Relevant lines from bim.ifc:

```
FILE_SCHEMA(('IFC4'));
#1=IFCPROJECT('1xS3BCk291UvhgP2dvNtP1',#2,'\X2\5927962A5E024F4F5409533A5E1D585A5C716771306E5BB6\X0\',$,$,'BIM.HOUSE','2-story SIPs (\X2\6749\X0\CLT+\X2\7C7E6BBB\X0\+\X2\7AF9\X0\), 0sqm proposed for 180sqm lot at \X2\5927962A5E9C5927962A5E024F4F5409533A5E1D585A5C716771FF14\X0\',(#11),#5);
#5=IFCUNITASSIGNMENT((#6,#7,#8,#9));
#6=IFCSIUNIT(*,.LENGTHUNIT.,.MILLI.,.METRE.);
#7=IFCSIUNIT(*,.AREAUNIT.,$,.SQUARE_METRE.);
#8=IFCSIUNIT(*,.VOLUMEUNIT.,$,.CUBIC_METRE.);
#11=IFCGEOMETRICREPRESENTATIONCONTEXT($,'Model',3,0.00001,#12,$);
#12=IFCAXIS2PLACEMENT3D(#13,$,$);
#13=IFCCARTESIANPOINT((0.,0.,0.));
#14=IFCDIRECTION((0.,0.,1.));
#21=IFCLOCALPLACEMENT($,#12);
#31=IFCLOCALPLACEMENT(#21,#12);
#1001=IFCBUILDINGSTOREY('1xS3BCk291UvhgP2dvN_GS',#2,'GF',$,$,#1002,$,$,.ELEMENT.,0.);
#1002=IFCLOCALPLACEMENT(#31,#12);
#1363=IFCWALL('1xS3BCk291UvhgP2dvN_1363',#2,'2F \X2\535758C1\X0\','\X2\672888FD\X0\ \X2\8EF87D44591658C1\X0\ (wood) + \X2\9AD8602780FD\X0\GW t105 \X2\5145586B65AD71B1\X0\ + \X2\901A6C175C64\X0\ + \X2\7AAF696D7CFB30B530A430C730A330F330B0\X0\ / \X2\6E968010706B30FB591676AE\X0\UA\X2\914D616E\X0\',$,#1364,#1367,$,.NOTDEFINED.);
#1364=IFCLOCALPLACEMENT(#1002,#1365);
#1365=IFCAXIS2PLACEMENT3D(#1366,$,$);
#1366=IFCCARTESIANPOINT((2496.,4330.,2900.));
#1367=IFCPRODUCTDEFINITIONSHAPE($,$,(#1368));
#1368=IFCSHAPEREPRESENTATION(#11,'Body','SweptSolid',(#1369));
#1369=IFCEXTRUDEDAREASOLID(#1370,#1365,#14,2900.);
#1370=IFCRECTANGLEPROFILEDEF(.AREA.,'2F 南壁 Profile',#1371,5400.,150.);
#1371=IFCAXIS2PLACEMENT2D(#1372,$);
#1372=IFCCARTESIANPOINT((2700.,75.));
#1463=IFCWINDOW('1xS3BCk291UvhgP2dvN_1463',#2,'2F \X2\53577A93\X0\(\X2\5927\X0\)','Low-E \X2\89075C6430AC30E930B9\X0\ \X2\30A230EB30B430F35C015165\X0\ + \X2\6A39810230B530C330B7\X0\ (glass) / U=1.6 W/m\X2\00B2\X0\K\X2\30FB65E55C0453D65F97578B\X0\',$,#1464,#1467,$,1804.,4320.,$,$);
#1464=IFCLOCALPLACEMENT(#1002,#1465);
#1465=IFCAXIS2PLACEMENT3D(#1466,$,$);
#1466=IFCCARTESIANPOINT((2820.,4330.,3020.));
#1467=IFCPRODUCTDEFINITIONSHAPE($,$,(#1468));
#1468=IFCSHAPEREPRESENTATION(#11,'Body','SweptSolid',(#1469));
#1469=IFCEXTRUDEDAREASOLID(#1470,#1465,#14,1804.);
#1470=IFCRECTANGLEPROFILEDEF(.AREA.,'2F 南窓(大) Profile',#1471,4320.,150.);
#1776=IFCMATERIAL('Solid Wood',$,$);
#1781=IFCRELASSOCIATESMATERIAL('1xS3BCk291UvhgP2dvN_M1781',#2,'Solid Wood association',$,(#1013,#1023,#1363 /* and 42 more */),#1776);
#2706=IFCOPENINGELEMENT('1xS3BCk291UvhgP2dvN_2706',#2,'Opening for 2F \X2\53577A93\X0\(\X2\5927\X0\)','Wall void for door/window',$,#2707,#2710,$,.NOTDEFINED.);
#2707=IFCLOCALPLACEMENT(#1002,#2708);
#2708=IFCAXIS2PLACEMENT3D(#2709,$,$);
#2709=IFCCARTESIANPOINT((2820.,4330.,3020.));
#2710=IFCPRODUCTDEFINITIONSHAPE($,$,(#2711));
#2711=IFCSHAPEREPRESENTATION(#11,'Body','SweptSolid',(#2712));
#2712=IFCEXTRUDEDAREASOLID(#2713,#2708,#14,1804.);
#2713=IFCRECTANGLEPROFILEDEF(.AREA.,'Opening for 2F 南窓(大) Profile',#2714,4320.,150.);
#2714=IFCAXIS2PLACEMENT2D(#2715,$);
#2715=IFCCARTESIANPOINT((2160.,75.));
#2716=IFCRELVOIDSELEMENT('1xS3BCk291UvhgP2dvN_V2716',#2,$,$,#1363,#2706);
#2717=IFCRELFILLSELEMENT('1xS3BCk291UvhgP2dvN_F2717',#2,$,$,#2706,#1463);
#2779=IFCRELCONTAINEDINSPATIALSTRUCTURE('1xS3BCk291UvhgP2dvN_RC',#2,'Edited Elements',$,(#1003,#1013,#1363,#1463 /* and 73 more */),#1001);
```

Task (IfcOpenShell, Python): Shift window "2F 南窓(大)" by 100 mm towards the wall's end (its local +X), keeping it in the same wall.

```python
import ifcopenshell
import ifcopenshell.api.geometry
import ifcopenshell.util.placement
import ifcopenshell.util.unit

model = ifcopenshell.open("bim.ifc")
unit_scale = ifcopenshell.util.unit.calculate_unit_scale(model)

window = model.by_guid("1xS3BCk291UvhgP2dvN_1463")
opening = window.FillsVoids[0].RelatingOpeningElement
wall = opening.VoidsElements[0].RelatingBuildingElement

wall_matrix = ifcopenshell.util.placement.get_local_placement(wall.ObjectPlacement)
shift = wall_matrix[:3, 0] * 0.1 / unit_scale
before = ifcopenshell.util.placement.get_local_placement(window.ObjectPlacement)[:3, 3].copy()

# The window is not placed relative to its opening, so move both.
for product in (opening, window):
    matrix = ifcopenshell.util.placement.get_local_placement(product.ObjectPlacement)
    matrix[:3, 3] += shift
    ifcopenshell.api.geometry.edit_object_placement(model, product=product, matrix=matrix, is_si=False)

after = ifcopenshell.util.placement.get_local_placement(window.ObjectPlacement)[:3, 3]
print("window moved by", (after - before).round(3) + 0.0)

model.write("bim-out.ifc")
```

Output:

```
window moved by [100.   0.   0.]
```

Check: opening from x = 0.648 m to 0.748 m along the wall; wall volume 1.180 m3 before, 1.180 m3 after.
